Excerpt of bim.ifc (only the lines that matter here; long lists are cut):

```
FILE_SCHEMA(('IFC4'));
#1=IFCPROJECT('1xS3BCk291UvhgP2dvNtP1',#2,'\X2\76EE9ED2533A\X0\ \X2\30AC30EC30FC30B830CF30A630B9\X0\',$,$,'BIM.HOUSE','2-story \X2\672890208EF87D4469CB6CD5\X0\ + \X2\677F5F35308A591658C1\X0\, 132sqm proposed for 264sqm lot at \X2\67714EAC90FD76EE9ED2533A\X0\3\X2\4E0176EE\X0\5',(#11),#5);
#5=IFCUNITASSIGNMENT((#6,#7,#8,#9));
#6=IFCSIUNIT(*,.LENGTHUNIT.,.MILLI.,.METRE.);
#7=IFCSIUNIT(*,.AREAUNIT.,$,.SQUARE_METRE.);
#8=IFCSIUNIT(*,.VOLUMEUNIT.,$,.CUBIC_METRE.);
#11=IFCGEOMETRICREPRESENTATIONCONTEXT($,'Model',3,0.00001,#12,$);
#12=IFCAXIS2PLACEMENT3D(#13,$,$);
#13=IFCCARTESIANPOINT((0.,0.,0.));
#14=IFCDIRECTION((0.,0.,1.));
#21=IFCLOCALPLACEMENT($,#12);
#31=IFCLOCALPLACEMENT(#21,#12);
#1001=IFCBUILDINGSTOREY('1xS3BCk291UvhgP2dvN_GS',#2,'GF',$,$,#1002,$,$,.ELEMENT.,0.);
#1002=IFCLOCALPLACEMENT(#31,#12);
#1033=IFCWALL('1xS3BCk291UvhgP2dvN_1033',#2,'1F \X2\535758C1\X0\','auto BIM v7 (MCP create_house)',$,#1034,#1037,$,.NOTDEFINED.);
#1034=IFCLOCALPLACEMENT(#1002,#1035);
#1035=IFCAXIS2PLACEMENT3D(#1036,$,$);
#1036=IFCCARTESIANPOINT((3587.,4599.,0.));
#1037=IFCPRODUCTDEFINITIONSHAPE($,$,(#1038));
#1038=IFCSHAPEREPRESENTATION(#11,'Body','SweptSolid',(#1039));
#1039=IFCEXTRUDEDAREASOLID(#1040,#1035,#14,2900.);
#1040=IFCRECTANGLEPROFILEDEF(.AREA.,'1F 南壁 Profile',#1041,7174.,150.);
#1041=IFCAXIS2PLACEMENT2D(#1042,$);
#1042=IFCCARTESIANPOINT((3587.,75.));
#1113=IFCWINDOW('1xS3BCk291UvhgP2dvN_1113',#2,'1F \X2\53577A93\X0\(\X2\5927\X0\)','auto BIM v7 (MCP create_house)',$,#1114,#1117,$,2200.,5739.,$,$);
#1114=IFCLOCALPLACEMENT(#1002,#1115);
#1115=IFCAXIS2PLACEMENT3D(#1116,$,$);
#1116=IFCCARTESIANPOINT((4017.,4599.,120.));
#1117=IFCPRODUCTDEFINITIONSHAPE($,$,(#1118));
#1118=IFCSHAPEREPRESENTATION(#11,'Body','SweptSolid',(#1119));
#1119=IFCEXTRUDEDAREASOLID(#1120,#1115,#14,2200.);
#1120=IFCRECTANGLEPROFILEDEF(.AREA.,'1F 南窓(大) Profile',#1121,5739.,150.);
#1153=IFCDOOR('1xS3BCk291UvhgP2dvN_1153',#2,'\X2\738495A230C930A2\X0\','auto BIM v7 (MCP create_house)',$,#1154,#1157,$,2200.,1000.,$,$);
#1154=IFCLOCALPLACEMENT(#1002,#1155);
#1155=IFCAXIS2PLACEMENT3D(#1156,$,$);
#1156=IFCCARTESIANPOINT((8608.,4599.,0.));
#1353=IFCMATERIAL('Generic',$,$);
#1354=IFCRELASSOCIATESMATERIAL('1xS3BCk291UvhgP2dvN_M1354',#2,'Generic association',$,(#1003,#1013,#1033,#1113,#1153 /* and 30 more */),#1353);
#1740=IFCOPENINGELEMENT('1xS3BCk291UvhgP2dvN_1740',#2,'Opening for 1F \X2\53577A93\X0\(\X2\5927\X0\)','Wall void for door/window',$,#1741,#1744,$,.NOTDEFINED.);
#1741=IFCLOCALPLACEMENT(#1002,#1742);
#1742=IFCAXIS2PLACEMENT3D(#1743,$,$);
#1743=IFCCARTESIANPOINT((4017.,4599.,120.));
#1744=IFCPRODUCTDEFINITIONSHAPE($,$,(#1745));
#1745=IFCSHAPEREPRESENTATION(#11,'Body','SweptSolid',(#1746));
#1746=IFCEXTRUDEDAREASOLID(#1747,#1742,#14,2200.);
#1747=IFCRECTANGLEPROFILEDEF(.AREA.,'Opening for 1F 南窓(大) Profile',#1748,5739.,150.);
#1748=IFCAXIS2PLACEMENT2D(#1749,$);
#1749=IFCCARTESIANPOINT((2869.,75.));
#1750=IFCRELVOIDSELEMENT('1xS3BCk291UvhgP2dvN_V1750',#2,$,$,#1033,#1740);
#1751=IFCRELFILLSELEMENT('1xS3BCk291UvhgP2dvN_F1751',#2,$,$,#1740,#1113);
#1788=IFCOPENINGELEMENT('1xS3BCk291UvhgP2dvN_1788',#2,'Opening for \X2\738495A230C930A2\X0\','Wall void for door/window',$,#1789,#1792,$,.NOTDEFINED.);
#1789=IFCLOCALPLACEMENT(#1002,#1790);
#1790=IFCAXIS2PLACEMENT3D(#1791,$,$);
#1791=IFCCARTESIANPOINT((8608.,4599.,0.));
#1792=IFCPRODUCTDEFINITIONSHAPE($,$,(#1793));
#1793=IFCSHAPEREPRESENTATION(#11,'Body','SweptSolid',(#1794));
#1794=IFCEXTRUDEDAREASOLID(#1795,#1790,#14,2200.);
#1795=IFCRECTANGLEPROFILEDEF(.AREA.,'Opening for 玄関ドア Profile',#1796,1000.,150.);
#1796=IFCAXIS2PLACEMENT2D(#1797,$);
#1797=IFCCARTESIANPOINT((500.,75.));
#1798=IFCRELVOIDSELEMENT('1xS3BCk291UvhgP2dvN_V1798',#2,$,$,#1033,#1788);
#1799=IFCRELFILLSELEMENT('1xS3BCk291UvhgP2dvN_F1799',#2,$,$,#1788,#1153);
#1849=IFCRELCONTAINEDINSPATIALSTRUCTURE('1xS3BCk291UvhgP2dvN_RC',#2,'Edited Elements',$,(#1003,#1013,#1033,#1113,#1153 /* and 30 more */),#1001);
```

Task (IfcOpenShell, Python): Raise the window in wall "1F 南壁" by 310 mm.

```python
import numpy as np
import ifcopenshell
import ifcopenshell.api.geometry
import ifcopenshell.util.placement
import ifcopenshell.util.unit

model = ifcopenshell.open("bim.ifc")
unit_scale = ifcopenshell.util.unit.calculate_unit_scale(model)

window = model.by_id(1113)
opening = window.FillsVoids[0].RelatingOpeningElement
dz = 0.31 / unit_scale

shift = np.array([0.0, 0.0, dz])
# The window is not placed relative to its opening, so move both.
for product in (opening, window):
    matrix = ifcopenshell.util.placement.get_local_placement(product.ObjectPlacement)
    matrix[:3, 3] += shift
    ifcopenshell.api.geometry.edit_object_placement(model, product=product, matrix=matrix, is_si=False)

print(f"moved by {dz * unit_scale:+.3f} m")

model.write("bim_rev.ifc")
```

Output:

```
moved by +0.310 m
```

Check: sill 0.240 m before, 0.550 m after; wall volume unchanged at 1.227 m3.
